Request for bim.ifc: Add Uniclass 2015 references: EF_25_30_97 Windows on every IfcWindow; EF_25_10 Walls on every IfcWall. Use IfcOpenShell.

First a look at what the model holds.

```python
import ifcopenshell

model = ifcopenshell.open("bim.ifc")
print(model.schema)
print("classifications:", [c.Name for c in model.by_type("IfcClassification")])
for ifc_class in ("IfcDoor", "IfcRoof", "IfcStair", "IfcWall", "IfcWindow"):
    print(ifc_class, len(model.by_type(ifc_class)))
```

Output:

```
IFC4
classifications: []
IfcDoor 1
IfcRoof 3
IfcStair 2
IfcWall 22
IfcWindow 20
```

```python
import ifcopenshell
import ifcopenshell.api.classification

model = ifcopenshell.open("bim.ifc")

system = ifcopenshell.api.classification.add_classification(model, classification="Uniclass 2015")

codes = {
    "IfcWindow": ("EF_25_30_97", "Windows"),
    "IfcWall": ("EF_25_10", "Walls"),
}
for ifc_class, (code, name) in codes.items():
    products = model.by_type(ifc_class)
    ifcopenshell.api.classification.add_reference(
        model, products=products, classification=system, identification=code, name=name
    )
    print(code, len(products))

model.write("bim-out.ifc")
```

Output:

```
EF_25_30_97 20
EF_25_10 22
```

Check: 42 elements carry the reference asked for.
